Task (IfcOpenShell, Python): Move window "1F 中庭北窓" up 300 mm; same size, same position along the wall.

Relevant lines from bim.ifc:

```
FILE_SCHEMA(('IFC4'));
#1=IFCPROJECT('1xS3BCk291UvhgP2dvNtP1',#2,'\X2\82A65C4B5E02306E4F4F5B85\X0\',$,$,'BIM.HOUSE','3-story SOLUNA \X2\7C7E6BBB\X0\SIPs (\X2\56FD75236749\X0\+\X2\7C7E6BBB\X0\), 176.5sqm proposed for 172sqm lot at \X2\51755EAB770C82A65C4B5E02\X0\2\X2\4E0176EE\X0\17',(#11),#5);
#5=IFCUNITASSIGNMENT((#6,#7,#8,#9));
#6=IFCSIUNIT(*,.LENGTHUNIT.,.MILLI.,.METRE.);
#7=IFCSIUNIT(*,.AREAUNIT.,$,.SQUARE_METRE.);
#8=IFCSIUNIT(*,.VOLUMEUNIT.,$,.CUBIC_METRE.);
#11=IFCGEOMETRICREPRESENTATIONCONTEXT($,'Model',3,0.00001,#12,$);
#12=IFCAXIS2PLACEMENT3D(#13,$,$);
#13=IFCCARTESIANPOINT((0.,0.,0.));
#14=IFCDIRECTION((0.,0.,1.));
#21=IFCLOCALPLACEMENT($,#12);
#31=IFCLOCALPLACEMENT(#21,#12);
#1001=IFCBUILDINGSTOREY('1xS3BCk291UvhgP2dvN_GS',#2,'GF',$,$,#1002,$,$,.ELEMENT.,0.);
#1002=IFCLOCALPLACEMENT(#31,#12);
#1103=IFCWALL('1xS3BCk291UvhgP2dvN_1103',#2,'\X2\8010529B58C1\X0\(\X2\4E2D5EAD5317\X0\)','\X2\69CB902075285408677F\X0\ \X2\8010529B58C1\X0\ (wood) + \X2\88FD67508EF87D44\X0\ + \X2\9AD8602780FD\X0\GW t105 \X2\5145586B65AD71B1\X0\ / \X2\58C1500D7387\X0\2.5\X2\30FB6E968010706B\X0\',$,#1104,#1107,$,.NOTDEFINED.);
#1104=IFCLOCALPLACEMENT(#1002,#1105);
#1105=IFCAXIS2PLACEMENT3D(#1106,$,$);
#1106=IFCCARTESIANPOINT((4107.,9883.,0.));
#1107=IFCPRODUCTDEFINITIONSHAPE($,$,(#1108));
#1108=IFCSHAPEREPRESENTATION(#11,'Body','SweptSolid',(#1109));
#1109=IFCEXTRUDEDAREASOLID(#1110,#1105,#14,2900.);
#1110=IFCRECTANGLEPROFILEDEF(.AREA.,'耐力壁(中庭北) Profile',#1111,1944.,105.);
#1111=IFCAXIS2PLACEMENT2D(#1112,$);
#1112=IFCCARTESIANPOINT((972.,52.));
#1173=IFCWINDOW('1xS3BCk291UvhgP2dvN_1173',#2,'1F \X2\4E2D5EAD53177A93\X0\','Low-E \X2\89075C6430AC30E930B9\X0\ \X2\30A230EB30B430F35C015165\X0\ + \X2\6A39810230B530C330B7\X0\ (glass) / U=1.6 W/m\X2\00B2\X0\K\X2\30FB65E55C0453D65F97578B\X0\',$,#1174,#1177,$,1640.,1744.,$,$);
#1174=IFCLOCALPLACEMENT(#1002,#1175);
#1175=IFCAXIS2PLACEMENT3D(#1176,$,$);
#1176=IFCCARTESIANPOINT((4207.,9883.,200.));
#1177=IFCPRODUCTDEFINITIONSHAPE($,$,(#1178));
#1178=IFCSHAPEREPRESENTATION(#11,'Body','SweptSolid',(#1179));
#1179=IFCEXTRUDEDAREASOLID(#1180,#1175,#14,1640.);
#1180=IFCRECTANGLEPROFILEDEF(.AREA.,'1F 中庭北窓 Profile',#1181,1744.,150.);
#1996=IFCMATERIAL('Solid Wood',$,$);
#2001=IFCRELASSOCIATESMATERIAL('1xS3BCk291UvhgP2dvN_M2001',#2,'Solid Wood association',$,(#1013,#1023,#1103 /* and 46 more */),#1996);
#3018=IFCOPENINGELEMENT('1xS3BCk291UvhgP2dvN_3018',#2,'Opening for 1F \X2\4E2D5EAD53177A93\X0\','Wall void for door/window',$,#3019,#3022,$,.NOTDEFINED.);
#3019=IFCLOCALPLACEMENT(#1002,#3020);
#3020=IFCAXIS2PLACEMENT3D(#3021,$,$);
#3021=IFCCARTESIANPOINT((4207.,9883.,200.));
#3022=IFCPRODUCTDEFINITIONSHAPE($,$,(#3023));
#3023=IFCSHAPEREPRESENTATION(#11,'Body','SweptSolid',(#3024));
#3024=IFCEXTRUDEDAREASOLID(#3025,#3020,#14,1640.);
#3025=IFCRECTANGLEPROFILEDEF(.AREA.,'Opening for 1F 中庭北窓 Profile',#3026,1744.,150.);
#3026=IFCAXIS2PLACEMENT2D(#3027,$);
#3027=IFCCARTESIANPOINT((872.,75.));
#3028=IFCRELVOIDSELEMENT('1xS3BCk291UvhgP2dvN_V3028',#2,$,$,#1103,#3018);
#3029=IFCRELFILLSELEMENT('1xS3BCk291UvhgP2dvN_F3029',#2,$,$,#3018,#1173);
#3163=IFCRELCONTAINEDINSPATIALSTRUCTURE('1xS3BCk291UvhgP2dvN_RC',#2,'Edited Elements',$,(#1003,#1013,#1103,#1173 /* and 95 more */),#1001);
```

```python
import numpy as np
import ifcopenshell
import ifcopenshell.api.geometry
import ifcopenshell.util.placement
import ifcopenshell.util.unit

model = ifcopenshell.open("bim.ifc")
unit_scale = ifcopenshell.util.unit.calculate_unit_scale(model)

window = model.by_guid("1xS3BCk291UvhgP2dvN_1173")
opening = window.FillsVoids[0].RelatingOpeningElement
dz = 300.0

shift = np.array([0.0, 0.0, dz])
# The window is not placed relative to its opening, so move both.
for product in (opening, window):
    matrix = ifcopenshell.util.placement.get_local_placement(product.ObjectPlacement)
    matrix[:3, 3] += shift
    ifcopenshell.api.geometry.edit_object_placement(model, product=product, matrix=matrix, is_si=False)

print(f"moved by {dz * unit_scale:+.3f} m")

model.write("bim_edited.ifc")
```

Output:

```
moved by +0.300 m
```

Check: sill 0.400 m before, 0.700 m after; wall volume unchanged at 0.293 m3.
